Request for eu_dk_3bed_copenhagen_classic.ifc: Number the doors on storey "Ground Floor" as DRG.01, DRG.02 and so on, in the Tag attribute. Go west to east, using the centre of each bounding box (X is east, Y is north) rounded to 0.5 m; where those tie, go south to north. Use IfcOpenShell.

First a look at what the model holds.

```python
import ifcopenshell
import ifcopenshell.util.element
import ifcopenshell.util.placement

model = ifcopenshell.open("eu_dk_3bed_copenhagen_classic.ifc")
print(model.schema)
storey = next(s for s in model.by_type("IfcBuildingStorey") if s.Name == "Ground Floor")
doors = [e for e in ifcopenshell.util.element.get_decomposition(storey) if e.is_a("IfcDoor")]
for e in sorted(doors, key=lambda e: e.id()):
    origin = ifcopenshell.util.placement.get_local_placement(e.ObjectPlacement)[:3, 3]
    print(e.id(), e.Tag, e.Name, origin.round(2) + 0.0, sep=" | ")
```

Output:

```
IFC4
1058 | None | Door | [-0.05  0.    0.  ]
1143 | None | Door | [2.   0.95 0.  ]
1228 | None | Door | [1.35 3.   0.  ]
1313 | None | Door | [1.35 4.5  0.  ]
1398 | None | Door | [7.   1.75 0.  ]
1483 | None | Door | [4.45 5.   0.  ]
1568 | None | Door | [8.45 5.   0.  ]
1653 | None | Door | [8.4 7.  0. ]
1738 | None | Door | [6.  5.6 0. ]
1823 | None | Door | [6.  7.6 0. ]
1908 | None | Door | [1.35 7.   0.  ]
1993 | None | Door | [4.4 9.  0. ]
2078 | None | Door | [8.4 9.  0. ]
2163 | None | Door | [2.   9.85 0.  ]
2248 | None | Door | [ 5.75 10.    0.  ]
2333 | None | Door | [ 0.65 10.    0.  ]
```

```python
import ifcopenshell
import ifcopenshell.geom
import ifcopenshell.util.element
import ifcopenshell.util.shape

model = ifcopenshell.open("eu_dk_3bed_copenhagen_classic.ifc")
settings = ifcopenshell.geom.settings()
settings.set("use-world-coords", True)


def centre(element):
    shape = ifcopenshell.geom.create_shape(settings, element)
    return ifcopenshell.util.shape.get_bbox_centroid(shape.geometry)


storey = next(s for s in model.by_type("IfcBuildingStorey") if s.Name == "Ground Floor")
doors = [e for e in ifcopenshell.util.element.get_decomposition(storey) if e.is_a("IfcDoor")]

# Insertion points can sit at a corner or the storey origin, so sort by the geometry (in metres).
centres = {e: centre(e) for e in doors}
doors.sort(key=lambda e: (round(centres[e][0] / 0.5), centres[e][1]))

for i, e in enumerate(doors, start=1):
    number = f"DRG.{i:02d}"
    e.Tag = number
    print(e.id(), number)

model.write("eu_dk_3bed_copenhagen_classic-out.ifc")
```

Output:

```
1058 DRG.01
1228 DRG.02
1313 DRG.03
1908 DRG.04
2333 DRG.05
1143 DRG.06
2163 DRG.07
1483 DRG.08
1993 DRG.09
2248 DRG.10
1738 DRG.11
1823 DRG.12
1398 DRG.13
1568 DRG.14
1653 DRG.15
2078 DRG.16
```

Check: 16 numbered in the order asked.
